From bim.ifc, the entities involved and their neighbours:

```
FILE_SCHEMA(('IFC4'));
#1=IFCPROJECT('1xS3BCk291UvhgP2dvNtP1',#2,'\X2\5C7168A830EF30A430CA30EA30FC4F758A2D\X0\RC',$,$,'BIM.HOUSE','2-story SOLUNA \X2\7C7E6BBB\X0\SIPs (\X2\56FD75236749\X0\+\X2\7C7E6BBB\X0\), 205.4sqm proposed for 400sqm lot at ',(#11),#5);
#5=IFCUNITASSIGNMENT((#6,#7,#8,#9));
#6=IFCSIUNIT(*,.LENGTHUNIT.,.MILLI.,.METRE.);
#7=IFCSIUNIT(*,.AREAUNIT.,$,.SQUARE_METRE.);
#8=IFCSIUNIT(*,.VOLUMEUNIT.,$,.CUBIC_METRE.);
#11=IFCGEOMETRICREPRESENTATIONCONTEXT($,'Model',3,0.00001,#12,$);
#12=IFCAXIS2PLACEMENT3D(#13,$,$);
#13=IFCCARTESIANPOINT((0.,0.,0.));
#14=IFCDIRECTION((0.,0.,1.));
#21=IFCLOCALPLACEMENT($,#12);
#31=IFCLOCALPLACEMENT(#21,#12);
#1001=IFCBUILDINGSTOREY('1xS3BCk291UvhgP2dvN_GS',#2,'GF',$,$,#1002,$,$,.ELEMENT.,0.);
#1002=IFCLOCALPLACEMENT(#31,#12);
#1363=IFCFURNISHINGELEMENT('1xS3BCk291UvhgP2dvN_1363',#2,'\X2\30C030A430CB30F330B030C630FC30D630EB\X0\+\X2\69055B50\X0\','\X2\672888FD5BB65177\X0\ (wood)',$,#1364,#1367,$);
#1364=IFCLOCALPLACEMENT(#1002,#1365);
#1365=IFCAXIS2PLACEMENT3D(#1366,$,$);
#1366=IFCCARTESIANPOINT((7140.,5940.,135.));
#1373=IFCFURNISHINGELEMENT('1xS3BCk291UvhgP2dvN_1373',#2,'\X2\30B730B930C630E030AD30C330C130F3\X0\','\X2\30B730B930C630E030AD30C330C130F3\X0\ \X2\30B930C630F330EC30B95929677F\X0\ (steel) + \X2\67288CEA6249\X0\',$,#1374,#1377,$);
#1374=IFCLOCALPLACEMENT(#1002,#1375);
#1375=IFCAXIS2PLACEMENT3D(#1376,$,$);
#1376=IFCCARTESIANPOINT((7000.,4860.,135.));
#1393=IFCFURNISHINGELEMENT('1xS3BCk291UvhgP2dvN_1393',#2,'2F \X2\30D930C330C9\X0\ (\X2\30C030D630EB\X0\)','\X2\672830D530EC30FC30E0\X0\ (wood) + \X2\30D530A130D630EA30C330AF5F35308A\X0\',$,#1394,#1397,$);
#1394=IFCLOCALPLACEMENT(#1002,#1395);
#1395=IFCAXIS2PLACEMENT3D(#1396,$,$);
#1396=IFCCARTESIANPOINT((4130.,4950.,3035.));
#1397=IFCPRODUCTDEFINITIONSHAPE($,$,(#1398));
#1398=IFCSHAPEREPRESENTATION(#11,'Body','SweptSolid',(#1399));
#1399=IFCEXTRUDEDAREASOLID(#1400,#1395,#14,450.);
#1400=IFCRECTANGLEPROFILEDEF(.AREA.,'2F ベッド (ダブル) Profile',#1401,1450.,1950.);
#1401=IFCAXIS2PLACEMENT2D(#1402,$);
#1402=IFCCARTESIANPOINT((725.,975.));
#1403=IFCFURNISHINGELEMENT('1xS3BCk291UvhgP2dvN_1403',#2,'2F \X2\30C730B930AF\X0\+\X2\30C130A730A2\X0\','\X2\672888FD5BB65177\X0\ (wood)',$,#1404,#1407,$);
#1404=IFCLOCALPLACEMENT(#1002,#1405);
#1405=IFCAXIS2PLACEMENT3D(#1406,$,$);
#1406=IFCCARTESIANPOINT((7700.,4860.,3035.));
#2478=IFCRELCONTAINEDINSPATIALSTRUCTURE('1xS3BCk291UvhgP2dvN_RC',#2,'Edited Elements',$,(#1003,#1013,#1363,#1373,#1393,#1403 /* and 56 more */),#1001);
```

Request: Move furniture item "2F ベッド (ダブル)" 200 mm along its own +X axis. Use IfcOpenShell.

```python
import ifcopenshell
import ifcopenshell.api.geometry
import ifcopenshell.util.placement
import ifcopenshell.util.unit

model = ifcopenshell.open("bim.ifc")
unit_scale = ifcopenshell.util.unit.calculate_unit_scale(model)

item = model.by_guid("1xS3BCk291UvhgP2dvN_1393")
matrix = ifcopenshell.util.placement.get_local_placement(item.ObjectPlacement)
matrix[:3, 3] += matrix[:3, 0] * 0.2 / unit_scale
ifcopenshell.api.geometry.edit_object_placement(model, product=item, matrix=matrix, is_si=False)

print(ifcopenshell.util.placement.get_local_placement(item.ObjectPlacement).round(3) + 0.0)

model.write("bim-out.ifc")
```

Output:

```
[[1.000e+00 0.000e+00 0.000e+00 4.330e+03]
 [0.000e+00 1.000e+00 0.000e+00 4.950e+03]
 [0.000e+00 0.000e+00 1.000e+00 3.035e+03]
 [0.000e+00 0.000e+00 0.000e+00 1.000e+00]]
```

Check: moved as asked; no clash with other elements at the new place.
